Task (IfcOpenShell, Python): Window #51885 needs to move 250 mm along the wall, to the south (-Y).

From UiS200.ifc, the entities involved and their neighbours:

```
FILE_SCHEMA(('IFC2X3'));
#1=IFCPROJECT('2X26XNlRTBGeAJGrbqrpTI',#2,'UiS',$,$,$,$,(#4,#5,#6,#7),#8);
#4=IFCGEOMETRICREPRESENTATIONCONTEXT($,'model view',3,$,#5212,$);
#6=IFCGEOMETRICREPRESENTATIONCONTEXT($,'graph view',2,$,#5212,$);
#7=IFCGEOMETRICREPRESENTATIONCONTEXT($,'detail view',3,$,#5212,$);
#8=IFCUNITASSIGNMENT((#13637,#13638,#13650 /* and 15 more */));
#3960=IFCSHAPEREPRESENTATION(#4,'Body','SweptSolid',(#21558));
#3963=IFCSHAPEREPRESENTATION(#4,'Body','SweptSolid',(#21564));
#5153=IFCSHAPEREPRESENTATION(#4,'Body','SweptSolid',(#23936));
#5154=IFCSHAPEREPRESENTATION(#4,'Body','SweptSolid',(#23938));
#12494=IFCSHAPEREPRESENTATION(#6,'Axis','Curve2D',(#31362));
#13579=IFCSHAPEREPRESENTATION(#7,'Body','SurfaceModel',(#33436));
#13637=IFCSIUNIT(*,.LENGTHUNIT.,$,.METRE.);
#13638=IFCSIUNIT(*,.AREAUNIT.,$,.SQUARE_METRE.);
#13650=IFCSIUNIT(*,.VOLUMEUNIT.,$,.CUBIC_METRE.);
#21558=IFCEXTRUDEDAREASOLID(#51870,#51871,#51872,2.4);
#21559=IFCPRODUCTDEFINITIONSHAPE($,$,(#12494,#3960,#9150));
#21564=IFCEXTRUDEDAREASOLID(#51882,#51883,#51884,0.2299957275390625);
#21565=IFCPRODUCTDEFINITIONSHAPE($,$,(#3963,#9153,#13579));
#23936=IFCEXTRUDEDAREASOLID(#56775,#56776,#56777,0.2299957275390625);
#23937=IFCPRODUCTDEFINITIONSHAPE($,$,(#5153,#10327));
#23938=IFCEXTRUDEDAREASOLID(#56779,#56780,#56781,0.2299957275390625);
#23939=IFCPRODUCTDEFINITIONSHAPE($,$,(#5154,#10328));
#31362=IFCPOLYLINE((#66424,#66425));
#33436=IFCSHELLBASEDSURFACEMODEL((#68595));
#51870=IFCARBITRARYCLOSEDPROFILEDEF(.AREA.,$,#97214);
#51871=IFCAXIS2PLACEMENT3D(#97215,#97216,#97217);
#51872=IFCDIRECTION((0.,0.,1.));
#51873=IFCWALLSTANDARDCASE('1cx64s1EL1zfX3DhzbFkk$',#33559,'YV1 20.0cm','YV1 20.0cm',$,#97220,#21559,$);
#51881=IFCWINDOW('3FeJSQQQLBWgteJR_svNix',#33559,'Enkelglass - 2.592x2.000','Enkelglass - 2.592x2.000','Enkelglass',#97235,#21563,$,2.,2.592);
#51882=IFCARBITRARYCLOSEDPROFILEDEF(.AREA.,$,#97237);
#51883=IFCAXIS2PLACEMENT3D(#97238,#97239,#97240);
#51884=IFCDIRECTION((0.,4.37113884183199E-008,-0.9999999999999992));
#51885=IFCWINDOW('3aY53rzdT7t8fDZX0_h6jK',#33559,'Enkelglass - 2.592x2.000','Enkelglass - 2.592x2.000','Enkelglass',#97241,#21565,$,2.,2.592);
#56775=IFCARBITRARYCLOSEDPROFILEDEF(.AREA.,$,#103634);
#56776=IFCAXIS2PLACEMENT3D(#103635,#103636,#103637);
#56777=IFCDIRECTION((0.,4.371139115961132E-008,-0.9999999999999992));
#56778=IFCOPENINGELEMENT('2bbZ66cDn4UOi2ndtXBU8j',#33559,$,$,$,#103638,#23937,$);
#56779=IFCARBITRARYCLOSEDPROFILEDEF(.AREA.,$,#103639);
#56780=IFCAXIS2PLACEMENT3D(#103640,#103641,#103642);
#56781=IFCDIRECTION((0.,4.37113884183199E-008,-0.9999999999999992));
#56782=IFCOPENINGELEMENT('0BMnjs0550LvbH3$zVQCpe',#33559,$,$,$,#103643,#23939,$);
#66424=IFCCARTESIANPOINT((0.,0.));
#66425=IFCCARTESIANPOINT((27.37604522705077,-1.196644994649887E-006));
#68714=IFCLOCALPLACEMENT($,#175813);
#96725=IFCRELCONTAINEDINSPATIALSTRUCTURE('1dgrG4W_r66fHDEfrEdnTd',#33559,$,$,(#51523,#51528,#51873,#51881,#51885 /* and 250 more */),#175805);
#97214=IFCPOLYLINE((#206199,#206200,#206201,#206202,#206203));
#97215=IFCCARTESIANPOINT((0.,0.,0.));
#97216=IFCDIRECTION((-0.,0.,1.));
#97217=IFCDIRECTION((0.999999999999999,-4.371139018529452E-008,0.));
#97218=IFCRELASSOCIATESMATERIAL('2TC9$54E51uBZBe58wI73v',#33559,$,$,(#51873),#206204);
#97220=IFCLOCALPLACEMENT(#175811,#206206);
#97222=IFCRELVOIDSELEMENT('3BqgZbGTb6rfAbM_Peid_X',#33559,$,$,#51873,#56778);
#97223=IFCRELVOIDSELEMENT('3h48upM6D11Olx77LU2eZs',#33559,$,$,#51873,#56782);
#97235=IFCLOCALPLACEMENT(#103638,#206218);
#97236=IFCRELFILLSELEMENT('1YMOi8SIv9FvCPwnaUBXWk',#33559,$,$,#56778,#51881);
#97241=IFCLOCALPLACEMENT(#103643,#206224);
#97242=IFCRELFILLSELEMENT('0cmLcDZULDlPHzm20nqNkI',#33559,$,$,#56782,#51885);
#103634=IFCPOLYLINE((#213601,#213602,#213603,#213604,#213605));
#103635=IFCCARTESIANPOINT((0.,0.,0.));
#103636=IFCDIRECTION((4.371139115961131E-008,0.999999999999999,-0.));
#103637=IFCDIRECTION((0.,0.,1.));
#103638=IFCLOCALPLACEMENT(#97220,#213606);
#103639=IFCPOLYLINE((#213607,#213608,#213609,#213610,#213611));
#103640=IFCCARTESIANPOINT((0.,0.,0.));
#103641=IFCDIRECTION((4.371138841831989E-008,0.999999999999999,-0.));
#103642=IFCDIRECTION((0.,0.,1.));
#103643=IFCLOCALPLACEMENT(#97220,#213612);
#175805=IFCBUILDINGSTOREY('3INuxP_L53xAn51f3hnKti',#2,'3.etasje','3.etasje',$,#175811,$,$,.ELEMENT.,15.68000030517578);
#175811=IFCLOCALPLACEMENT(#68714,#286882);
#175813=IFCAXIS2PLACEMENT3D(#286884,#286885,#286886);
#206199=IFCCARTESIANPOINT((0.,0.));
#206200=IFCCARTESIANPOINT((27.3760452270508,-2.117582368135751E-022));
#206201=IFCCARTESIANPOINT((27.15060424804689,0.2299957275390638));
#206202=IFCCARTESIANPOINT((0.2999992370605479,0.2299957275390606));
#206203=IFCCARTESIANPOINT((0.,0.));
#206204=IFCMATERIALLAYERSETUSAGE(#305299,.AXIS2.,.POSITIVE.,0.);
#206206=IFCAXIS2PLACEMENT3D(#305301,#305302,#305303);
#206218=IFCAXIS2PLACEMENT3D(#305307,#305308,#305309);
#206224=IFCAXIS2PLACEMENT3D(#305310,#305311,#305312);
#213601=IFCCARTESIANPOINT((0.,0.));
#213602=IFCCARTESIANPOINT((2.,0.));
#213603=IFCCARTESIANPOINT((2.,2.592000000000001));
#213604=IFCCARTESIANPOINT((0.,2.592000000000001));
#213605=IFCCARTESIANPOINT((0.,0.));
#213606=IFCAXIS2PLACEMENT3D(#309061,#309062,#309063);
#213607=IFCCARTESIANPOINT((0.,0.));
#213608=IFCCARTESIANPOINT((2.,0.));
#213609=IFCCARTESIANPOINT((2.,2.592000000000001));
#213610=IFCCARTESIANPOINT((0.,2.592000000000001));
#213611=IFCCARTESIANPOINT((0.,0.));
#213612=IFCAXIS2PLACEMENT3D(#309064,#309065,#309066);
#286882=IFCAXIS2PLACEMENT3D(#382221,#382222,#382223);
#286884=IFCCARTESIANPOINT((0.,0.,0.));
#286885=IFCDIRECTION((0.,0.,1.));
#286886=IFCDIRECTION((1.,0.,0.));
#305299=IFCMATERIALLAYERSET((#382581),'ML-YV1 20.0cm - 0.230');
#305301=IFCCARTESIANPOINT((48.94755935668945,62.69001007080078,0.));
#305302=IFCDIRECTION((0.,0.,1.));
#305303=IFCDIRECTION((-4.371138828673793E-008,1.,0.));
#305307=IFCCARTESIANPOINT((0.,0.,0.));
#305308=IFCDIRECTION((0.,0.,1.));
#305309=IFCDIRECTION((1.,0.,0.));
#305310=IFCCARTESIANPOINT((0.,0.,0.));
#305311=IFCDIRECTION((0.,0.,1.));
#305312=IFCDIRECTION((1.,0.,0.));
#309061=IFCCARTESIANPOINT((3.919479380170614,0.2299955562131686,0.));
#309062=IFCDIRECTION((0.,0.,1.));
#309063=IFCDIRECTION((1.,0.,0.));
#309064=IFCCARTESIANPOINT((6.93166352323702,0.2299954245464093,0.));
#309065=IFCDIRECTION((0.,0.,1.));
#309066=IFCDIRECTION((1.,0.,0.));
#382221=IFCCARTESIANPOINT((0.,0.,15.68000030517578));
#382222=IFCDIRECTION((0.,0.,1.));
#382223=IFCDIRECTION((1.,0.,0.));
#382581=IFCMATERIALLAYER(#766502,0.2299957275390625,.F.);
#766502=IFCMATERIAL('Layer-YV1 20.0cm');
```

```python
import ifcopenshell
import ifcopenshell.api.geometry
import ifcopenshell.util.placement

model = ifcopenshell.open("UiS200.ifc")

window = model.by_guid("3aY53rzdT7t8fDZX0_h6jK")
opening = window.FillsVoids[0].RelatingOpeningElement
wall = opening.VoidsElements[0].RelatingBuildingElement

wall_matrix = ifcopenshell.util.placement.get_local_placement(wall.ObjectPlacement)
shift = wall_matrix[:3, 0] * -0.25
before = ifcopenshell.util.placement.get_local_placement(window.ObjectPlacement)[:3, 3].copy()

# The window is placed relative to its opening, so it follows when the opening moves.
matrix = ifcopenshell.util.placement.get_local_placement(opening.ObjectPlacement)
matrix[:3, 3] += shift
ifcopenshell.api.geometry.edit_object_placement(
    model, product=opening, matrix=matrix, is_si=False, should_transform_children=True
)

after = ifcopenshell.util.placement.get_local_placement(window.ObjectPlacement)[:3, 3]
print("window moved by", (after - before).round(3) + 0.0)

model.write("UiS200_v2.ifc")
```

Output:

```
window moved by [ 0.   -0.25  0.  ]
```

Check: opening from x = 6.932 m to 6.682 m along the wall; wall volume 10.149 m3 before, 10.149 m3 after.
